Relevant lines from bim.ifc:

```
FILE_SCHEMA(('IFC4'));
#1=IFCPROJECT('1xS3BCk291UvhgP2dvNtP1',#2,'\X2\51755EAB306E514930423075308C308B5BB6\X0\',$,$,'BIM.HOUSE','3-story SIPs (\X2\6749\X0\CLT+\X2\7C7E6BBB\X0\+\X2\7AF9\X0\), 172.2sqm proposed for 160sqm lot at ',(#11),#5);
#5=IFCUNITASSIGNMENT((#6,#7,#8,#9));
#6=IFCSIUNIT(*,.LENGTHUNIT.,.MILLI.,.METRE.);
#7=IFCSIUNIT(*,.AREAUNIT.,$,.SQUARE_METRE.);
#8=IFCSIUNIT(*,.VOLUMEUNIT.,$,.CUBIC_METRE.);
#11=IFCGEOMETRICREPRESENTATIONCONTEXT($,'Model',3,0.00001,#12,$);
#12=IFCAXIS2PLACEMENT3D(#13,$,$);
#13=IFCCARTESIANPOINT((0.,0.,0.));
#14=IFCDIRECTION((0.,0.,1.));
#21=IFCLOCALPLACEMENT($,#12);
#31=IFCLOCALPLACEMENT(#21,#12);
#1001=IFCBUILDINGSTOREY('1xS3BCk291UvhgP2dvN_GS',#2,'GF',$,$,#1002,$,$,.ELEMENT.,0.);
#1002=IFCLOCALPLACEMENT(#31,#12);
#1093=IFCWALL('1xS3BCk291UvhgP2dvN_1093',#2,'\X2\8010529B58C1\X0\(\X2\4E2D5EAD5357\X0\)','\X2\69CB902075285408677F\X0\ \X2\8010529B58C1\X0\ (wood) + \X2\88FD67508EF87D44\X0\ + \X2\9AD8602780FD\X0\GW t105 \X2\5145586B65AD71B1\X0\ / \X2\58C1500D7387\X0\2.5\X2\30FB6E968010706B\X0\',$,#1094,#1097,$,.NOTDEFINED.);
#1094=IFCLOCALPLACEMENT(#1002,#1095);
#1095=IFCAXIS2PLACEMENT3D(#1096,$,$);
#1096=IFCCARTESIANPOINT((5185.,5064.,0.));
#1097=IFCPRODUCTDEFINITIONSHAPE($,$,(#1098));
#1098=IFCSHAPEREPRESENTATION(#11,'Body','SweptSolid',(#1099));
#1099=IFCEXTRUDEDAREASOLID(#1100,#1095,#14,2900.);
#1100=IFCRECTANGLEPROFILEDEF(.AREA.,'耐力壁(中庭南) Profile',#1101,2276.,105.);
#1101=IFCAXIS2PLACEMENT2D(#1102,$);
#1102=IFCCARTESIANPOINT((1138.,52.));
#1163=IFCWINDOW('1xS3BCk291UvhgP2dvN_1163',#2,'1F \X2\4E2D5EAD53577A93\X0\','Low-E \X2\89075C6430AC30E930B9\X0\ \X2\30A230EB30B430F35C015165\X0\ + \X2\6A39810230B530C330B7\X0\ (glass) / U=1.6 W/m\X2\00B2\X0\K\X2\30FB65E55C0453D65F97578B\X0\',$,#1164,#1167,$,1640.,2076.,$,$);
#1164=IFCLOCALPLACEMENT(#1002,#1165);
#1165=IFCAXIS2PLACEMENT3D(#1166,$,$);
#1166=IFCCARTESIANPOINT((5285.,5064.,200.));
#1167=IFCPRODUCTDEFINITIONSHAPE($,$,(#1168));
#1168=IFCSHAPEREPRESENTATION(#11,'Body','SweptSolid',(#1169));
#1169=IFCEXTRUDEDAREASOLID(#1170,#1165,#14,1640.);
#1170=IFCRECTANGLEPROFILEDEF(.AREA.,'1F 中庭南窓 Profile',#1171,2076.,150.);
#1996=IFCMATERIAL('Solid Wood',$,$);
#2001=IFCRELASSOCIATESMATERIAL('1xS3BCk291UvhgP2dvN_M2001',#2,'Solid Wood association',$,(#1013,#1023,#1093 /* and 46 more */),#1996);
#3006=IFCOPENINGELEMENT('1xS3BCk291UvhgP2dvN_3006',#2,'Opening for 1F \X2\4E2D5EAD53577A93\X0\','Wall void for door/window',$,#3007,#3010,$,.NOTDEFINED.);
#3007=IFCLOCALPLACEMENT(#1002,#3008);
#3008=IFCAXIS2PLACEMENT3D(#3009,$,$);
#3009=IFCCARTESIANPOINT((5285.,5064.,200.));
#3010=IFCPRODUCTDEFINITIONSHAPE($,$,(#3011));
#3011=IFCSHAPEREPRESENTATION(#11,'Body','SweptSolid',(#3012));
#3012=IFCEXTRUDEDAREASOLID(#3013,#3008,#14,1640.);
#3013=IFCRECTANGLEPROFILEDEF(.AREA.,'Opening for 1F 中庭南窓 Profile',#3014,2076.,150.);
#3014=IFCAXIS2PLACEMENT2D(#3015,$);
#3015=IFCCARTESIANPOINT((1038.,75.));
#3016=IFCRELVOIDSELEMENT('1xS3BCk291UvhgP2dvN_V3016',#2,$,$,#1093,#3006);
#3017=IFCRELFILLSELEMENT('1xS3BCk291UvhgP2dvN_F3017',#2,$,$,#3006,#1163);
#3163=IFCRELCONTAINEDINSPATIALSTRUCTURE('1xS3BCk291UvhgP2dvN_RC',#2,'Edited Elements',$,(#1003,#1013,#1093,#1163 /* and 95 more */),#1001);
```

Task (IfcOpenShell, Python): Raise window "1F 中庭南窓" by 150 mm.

```python
import numpy as np
import ifcopenshell
import ifcopenshell.api.geometry
import ifcopenshell.util.placement
import ifcopenshell.util.unit

model = ifcopenshell.open("bim.ifc")
unit_scale = ifcopenshell.util.unit.calculate_unit_scale(model)

window = model.by_id(1163)
opening = window.FillsVoids[0].RelatingOpeningElement
dz = 0.15 / unit_scale

shift = np.array([0.0, 0.0, dz])
# The window is not placed relative to its opening, so move both.
for product in (opening, window):
    matrix = ifcopenshell.util.placement.get_local_placement(product.ObjectPlacement)
    matrix[:3, 3] += shift
    ifcopenshell.api.geometry.edit_object_placement(model, product=product, matrix=matrix, is_si=False)

print(f"moved by {dz * unit_scale:+.3f} m")

model.write("bim-out.ifc")
```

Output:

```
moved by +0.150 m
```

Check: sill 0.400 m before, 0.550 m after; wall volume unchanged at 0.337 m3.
